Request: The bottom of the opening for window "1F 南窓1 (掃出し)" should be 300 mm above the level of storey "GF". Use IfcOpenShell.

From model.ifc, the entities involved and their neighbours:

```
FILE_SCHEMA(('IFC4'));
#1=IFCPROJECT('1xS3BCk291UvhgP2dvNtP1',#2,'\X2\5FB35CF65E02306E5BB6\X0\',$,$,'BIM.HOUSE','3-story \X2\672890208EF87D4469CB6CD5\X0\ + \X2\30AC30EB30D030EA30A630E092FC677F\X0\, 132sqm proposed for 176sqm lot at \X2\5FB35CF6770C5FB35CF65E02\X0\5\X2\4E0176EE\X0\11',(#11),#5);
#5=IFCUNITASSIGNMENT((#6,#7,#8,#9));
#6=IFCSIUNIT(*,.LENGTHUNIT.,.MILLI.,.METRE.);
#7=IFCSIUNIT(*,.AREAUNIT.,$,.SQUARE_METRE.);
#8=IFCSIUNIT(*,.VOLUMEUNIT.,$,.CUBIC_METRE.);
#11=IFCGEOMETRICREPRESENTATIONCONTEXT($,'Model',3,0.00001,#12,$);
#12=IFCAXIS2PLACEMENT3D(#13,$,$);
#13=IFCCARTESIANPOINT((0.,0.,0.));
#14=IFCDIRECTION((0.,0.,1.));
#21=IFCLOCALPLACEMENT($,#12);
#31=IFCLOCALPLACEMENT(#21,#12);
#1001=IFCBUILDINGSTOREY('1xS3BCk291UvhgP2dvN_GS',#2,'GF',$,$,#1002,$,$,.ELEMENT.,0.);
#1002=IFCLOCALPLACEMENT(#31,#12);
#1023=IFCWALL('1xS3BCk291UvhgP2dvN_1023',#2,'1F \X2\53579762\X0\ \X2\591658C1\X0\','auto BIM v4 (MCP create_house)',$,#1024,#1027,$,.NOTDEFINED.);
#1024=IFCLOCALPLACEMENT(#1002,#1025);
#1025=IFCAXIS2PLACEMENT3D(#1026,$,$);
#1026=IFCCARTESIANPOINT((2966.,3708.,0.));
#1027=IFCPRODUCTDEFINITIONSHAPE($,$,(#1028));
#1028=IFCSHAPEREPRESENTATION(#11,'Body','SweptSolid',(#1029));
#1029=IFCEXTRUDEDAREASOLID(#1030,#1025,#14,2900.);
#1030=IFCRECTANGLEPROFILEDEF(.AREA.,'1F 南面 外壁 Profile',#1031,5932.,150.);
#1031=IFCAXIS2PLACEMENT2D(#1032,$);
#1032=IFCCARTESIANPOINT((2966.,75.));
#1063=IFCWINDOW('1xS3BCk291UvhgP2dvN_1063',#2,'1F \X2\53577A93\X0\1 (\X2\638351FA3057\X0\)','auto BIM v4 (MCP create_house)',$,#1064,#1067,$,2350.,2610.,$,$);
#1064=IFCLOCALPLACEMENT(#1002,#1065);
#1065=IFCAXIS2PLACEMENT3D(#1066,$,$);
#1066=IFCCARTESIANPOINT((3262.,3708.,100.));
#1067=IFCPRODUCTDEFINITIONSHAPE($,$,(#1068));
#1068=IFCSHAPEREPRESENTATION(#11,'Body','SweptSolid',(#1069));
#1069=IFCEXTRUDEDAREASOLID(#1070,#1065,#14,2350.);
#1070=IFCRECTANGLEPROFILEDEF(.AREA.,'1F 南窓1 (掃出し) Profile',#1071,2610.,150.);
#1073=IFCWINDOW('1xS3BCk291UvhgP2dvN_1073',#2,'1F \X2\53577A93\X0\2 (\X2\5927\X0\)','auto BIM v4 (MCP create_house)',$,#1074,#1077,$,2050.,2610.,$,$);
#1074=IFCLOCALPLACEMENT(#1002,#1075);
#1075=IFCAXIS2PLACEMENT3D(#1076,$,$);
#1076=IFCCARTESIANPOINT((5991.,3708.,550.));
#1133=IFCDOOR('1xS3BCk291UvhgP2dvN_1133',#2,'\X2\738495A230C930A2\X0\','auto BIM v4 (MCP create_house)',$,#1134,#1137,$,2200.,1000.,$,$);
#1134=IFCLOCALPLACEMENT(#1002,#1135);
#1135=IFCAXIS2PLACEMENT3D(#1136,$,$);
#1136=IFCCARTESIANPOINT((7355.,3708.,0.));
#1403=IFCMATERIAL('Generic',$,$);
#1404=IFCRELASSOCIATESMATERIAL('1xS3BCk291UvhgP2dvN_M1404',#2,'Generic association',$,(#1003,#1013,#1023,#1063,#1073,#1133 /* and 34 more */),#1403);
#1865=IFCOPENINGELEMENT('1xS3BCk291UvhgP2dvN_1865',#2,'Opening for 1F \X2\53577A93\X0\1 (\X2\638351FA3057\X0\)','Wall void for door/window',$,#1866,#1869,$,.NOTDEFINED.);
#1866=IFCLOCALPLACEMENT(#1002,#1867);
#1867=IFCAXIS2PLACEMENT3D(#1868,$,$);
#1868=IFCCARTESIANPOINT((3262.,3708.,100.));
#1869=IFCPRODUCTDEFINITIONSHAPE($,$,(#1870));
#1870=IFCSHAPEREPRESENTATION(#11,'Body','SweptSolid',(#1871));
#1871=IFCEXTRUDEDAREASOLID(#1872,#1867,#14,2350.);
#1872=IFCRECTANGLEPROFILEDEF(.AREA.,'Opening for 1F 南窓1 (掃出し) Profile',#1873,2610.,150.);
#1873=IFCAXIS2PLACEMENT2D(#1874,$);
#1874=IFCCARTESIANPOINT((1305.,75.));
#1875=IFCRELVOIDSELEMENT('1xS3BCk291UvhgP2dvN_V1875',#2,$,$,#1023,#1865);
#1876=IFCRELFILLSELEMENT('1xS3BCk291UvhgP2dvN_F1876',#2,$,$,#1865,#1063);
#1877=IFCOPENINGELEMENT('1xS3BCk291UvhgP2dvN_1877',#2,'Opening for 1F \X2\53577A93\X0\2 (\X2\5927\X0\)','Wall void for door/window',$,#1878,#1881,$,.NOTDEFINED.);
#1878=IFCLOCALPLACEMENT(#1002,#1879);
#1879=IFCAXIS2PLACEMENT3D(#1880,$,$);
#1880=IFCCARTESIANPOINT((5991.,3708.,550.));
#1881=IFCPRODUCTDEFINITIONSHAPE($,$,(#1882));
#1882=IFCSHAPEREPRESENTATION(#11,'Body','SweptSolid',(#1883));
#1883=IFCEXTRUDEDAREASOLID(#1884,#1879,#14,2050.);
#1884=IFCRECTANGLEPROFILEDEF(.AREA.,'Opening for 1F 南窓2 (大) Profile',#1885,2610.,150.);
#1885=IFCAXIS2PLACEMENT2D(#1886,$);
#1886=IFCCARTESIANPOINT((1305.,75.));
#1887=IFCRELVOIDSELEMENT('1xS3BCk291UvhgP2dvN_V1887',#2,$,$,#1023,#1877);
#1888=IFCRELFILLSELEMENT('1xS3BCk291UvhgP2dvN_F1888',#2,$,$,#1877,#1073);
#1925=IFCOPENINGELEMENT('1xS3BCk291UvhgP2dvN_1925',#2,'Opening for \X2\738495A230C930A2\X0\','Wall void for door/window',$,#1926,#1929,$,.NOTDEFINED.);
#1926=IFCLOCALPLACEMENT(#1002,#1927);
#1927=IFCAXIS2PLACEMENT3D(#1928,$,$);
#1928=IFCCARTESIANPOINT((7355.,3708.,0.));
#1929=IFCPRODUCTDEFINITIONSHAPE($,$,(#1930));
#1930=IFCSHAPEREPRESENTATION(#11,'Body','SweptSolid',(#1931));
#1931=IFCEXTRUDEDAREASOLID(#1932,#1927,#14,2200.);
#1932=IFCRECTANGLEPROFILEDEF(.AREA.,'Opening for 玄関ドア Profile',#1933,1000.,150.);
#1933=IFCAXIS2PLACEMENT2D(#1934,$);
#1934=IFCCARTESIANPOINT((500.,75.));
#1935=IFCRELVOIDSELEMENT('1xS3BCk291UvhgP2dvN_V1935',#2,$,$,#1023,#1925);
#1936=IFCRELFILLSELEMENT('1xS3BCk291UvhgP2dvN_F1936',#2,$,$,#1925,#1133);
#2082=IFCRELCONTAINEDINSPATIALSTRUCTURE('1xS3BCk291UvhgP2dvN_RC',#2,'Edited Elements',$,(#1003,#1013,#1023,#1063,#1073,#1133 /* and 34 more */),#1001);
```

```python
import numpy as np
import ifcopenshell
import ifcopenshell.api.geometry
import ifcopenshell.geom
import ifcopenshell.util.element
import ifcopenshell.util.placement
import ifcopenshell.util.shape
import ifcopenshell.util.unit

model = ifcopenshell.open("model.ifc")
unit_scale = ifcopenshell.util.unit.calculate_unit_scale(model)

window = model.by_guid("1xS3BCk291UvhgP2dvN_1063")
opening = window.FillsVoids[0].RelatingOpeningElement
storey = ifcopenshell.util.element.get_container(window, ifc_class="IfcBuildingStorey")
level = ifcopenshell.util.placement.get_local_placement(storey.ObjectPlacement)[2, 3]

# The opening's origin need not be at the sill, so measure its lowest point.
shape = ifcopenshell.geom.create_shape(ifcopenshell.geom.settings(), opening)
bottom = ifcopenshell.util.shape.get_shape_bottom_elevation(shape, shape.geometry) / unit_scale
dz = level + 0.3 / unit_scale - bottom

shift = np.array([0.0, 0.0, dz])
# The window is not placed relative to its opening, so move both.
for product in (opening, window):
    matrix = ifcopenshell.util.placement.get_local_placement(product.ObjectPlacement)
    matrix[:3, 3] += shift
    ifcopenshell.api.geometry.edit_object_placement(model, product=product, matrix=matrix, is_si=False)

print(f"moved by {dz * unit_scale:+.3f} m")

model.write("model-out.ifc")
```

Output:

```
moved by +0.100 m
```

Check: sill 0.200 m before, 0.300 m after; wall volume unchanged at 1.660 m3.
